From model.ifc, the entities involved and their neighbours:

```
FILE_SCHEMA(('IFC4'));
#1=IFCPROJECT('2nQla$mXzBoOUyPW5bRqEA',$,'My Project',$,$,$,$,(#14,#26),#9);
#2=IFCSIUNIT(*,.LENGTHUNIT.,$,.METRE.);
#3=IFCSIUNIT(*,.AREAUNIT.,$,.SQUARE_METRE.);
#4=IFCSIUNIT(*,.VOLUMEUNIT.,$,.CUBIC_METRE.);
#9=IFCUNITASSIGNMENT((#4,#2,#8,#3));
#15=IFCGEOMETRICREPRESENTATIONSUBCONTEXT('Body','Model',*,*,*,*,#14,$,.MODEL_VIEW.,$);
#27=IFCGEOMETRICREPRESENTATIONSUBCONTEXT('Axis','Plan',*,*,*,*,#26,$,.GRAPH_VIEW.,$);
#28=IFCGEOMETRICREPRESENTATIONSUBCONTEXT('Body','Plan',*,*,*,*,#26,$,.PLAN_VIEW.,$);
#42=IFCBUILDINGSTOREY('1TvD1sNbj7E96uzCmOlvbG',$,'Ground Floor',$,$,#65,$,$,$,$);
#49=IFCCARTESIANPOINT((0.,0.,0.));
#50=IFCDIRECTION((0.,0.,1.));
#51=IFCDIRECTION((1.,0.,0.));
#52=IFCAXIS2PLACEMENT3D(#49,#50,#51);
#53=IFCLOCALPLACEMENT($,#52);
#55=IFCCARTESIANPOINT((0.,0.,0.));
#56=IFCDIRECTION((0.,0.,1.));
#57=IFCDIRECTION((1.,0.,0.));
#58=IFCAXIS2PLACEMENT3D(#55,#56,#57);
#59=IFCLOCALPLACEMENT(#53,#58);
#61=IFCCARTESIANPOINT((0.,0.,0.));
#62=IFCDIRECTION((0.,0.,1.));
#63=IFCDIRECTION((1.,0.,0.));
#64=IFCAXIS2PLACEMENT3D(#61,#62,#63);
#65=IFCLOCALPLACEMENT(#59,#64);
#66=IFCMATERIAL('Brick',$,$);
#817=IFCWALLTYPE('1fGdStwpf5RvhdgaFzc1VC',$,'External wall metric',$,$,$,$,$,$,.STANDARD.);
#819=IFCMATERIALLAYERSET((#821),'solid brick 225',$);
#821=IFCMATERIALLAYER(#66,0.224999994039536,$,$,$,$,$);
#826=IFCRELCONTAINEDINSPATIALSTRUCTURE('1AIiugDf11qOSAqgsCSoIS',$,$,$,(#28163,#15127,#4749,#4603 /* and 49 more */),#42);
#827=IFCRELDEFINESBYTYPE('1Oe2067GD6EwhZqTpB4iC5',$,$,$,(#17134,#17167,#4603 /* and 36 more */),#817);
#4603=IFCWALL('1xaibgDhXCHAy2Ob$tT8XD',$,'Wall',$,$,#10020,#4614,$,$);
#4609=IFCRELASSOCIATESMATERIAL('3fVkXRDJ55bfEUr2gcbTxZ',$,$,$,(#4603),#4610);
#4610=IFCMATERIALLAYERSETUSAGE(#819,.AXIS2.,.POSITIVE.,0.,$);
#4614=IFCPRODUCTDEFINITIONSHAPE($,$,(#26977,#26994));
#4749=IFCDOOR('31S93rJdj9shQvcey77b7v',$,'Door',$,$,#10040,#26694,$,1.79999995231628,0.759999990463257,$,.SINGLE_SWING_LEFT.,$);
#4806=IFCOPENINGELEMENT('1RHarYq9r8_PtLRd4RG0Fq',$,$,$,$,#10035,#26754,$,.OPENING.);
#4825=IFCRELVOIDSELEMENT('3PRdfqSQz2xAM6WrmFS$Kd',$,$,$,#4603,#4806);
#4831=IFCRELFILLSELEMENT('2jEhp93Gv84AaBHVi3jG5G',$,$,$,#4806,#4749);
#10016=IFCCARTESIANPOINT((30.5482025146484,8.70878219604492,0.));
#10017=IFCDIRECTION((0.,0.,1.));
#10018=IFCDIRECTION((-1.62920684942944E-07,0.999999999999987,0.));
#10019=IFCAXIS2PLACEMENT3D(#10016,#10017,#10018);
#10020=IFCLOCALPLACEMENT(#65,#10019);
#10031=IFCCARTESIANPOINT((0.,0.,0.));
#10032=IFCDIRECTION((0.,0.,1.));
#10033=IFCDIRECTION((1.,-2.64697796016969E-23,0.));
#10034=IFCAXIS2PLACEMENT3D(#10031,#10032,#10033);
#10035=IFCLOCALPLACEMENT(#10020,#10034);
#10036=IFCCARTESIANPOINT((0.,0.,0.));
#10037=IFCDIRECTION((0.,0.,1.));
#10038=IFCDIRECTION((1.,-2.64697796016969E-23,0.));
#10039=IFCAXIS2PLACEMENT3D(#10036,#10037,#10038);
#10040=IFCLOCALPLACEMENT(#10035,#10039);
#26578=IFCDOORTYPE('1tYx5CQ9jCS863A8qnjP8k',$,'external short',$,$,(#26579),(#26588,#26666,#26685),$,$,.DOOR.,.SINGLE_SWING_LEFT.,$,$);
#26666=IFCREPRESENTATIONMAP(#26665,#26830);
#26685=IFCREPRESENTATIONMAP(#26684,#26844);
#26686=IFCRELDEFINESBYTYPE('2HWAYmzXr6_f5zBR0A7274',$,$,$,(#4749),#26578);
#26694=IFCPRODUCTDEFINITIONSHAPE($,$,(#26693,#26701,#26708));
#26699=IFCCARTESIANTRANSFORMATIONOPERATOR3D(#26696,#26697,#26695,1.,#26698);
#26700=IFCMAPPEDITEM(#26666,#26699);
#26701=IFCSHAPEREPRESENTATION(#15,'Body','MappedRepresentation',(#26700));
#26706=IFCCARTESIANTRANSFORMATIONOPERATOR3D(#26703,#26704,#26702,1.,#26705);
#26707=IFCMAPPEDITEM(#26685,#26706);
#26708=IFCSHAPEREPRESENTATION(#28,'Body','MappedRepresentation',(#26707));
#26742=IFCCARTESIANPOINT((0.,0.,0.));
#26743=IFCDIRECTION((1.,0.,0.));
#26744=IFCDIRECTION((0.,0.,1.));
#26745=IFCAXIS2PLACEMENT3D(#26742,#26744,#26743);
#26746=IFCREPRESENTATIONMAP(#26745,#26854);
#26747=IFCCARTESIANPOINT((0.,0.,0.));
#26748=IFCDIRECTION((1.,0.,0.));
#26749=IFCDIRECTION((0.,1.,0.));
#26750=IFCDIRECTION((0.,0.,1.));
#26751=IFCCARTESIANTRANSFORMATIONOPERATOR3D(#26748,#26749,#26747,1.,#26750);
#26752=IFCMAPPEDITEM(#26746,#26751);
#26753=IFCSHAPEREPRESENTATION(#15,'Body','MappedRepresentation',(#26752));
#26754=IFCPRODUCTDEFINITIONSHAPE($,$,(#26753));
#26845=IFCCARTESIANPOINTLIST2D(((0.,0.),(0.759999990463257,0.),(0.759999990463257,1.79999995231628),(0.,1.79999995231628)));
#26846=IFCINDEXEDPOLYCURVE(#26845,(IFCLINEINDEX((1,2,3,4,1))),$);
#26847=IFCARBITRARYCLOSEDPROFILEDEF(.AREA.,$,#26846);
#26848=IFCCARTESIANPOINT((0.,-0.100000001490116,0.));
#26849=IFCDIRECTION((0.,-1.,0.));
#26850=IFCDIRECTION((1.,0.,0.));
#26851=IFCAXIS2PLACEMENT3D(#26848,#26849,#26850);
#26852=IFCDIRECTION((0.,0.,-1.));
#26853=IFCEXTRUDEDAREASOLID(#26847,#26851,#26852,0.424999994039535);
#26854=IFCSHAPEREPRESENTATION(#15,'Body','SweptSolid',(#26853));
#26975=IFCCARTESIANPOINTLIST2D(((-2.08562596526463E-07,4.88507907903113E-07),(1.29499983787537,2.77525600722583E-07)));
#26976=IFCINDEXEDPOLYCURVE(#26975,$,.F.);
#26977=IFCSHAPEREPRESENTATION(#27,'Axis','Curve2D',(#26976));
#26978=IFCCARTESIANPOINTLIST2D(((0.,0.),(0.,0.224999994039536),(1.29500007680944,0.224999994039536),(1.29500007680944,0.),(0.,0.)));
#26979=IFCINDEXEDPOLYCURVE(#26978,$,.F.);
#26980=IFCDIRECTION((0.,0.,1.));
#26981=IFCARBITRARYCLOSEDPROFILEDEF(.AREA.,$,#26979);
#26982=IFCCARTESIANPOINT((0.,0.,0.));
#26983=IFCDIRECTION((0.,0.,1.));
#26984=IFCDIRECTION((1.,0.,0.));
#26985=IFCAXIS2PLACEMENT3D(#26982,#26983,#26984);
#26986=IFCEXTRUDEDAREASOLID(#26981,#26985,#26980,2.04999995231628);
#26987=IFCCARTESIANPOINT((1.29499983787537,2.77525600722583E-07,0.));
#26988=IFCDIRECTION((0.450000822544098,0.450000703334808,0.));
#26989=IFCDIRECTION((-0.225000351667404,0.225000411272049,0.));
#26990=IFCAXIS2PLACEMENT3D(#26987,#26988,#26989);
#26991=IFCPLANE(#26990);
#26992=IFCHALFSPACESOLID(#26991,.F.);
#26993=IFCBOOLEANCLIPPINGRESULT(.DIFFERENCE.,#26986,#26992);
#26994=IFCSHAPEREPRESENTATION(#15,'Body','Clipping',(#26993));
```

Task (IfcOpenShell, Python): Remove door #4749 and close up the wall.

```python
import ifcopenshell
import ifcopenshell.api.feature
import ifcopenshell.api.root
import ifcopenshell.geom
import ifcopenshell.util.shape

model = ifcopenshell.open("model.ifc")
settings = ifcopenshell.geom.settings()


def volume(element):
    """Net volume in cubic metres, openings subtracted."""
    shape = ifcopenshell.geom.create_shape(settings, element)
    return ifcopenshell.util.shape.get_volume(shape.geometry)


door = model.by_guid("31S93rJdj9shQvcey77b7v")
opening = door.FillsVoids[0].RelatingOpeningElement
wall = opening.VoidsElements[0].RelatingBuildingElement
before = volume(wall)

ifcopenshell.api.root.remove_product(model, product=door)
ifcopenshell.api.feature.remove_feature(model, feature=opening)

after = volume(wall)

print(f"wall volume {before:.3f} -> {after:.3f} m3")

model.write("model_rev.ifc")
```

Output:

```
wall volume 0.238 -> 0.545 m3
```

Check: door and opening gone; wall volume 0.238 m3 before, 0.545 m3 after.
